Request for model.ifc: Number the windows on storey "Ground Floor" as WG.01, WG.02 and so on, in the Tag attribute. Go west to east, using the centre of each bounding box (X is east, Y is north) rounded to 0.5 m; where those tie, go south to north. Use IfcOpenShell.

First a look at what the model holds.

```python
import ifcopenshell
import ifcopenshell.util.element
import ifcopenshell.util.placement

model = ifcopenshell.open("model.ifc")
print(model.schema)
storey = next(s for s in model.by_type("IfcBuildingStorey") if s.Name == "Ground Floor")
windows = [e for e in ifcopenshell.util.element.get_decomposition(storey) if e.is_a("IfcWindow")]
for e in sorted(windows, key=lambda e: e.id()):
    origin = ifcopenshell.util.placement.get_local_placement(e.ObjectPlacement)[:3, 3]
    print(e.id(), e.Tag, e.Name, origin.round(2) + 0.0, sep=" | ")
```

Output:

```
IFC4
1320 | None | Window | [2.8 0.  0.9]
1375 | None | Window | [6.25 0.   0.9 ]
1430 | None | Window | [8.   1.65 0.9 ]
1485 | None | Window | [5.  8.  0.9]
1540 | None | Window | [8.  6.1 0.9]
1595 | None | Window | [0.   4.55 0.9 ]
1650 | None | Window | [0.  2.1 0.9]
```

```python
import ifcopenshell
import ifcopenshell.geom
import ifcopenshell.util.element
import ifcopenshell.util.shape

model = ifcopenshell.open("model.ifc")
settings = ifcopenshell.geom.settings()
settings.set("use-world-coords", True)


def centre(element):
    shape = ifcopenshell.geom.create_shape(settings, element)
    return ifcopenshell.util.shape.get_bbox_centroid(shape.geometry)


storey = next(s for s in model.by_type("IfcBuildingStorey") if s.Name == "Ground Floor")
windows = [e for e in ifcopenshell.util.element.get_decomposition(storey) if e.is_a("IfcWindow")]

# Insertion points can sit at a corner or the storey origin, so sort by the geometry (in metres).
centres = {e: centre(e) for e in windows}
windows.sort(key=lambda e: (round(centres[e][0] / 0.5), centres[e][1]))

for i, e in enumerate(windows, start=1):
    number = f"WG.{i:02d}"
    e.Tag = number
    print(e.id(), number)

model.write("model_rev.ifc")
```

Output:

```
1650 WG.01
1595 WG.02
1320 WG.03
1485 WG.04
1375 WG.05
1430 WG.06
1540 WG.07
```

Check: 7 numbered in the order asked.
